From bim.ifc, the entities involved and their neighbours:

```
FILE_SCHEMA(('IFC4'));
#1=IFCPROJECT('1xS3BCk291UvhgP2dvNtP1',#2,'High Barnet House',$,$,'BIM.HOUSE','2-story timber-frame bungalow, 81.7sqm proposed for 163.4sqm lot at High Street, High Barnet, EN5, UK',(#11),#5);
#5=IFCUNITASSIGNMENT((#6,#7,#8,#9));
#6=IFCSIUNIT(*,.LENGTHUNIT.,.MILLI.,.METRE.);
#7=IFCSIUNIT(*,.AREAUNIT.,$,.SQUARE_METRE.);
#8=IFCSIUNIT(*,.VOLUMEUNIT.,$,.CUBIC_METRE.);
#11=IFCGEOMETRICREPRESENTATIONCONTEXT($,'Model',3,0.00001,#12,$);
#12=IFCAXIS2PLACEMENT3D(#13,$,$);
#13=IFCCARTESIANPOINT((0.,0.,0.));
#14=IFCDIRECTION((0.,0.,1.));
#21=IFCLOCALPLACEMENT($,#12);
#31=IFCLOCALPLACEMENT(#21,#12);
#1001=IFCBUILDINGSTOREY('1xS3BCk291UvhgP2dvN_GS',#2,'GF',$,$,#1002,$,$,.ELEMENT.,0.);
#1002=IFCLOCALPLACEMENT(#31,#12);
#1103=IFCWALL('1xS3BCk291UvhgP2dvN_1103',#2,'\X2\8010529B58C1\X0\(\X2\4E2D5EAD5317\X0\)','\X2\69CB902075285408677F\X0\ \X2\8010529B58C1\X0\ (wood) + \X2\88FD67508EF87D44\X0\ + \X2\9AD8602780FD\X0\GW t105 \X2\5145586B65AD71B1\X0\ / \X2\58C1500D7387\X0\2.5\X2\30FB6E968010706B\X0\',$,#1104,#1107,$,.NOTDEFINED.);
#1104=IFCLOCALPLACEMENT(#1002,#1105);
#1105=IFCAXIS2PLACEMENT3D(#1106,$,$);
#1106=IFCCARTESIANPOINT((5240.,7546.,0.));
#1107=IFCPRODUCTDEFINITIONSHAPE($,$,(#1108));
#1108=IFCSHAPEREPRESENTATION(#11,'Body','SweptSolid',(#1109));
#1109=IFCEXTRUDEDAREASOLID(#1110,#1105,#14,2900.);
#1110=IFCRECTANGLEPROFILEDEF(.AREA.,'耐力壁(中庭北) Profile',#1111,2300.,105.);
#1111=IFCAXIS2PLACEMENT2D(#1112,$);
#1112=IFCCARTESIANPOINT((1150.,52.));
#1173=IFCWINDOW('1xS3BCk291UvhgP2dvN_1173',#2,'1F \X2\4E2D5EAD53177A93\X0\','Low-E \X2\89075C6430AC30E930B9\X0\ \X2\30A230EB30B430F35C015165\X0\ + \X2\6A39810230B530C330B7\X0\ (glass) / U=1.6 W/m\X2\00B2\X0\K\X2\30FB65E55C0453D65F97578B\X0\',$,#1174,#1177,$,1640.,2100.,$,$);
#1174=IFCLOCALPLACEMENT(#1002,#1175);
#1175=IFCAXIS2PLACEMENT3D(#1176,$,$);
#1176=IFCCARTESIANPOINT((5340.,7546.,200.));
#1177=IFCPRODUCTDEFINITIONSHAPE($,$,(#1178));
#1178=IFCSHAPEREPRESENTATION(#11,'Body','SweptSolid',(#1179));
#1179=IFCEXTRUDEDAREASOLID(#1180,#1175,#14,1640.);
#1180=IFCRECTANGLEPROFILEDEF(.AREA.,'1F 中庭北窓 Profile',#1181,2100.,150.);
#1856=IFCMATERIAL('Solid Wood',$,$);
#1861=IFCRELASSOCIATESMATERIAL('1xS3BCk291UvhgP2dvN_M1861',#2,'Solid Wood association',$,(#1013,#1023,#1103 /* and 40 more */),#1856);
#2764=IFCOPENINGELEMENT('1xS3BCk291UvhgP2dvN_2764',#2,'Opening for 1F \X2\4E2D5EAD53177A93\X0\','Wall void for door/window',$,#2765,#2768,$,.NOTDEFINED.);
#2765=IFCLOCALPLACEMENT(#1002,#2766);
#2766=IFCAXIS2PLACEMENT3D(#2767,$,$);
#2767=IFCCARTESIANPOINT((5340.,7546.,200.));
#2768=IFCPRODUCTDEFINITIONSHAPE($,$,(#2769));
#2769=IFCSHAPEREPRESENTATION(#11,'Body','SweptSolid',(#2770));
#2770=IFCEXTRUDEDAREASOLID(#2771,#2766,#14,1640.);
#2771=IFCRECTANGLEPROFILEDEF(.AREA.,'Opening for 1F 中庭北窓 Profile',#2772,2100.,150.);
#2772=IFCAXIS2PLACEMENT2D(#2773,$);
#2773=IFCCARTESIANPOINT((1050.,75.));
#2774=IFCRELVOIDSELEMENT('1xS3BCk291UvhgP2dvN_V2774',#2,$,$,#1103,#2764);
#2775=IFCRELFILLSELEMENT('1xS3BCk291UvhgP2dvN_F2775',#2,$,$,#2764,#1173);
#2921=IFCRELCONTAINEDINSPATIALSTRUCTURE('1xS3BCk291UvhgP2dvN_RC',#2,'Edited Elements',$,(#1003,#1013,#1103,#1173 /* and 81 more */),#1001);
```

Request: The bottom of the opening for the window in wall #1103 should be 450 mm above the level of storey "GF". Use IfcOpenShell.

```python
import numpy as np
import ifcopenshell
import ifcopenshell.api.geometry
import ifcopenshell.geom
import ifcopenshell.util.element
import ifcopenshell.util.placement
import ifcopenshell.util.shape
import ifcopenshell.util.unit

model = ifcopenshell.open("bim.ifc")
unit_scale = ifcopenshell.util.unit.calculate_unit_scale(model)

window = model.by_guid("1xS3BCk291UvhgP2dvN_1173")
opening = window.FillsVoids[0].RelatingOpeningElement
storey = ifcopenshell.util.element.get_container(window, ifc_class="IfcBuildingStorey")
level = ifcopenshell.util.placement.get_local_placement(storey.ObjectPlacement)[2, 3]

# The opening's origin need not be at the sill, so measure its lowest point.
shape = ifcopenshell.geom.create_shape(ifcopenshell.geom.settings(), opening)
bottom = ifcopenshell.util.shape.get_shape_bottom_elevation(shape, shape.geometry) / unit_scale
dz = level + 0.45 / unit_scale - bottom

shift = np.array([0.0, 0.0, dz])
# The window is not placed relative to its opening, so move both.
for product in (opening, window):
    matrix = ifcopenshell.util.placement.get_local_placement(product.ObjectPlacement)
    matrix[:3, 3] += shift
    ifcopenshell.api.geometry.edit_object_placement(model, product=product, matrix=matrix, is_si=False)

print(f"moved by {dz * unit_scale:+.3f} m")

model.write("bim_updated.ifc")
```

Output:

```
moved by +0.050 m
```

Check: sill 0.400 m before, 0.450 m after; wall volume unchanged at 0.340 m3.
